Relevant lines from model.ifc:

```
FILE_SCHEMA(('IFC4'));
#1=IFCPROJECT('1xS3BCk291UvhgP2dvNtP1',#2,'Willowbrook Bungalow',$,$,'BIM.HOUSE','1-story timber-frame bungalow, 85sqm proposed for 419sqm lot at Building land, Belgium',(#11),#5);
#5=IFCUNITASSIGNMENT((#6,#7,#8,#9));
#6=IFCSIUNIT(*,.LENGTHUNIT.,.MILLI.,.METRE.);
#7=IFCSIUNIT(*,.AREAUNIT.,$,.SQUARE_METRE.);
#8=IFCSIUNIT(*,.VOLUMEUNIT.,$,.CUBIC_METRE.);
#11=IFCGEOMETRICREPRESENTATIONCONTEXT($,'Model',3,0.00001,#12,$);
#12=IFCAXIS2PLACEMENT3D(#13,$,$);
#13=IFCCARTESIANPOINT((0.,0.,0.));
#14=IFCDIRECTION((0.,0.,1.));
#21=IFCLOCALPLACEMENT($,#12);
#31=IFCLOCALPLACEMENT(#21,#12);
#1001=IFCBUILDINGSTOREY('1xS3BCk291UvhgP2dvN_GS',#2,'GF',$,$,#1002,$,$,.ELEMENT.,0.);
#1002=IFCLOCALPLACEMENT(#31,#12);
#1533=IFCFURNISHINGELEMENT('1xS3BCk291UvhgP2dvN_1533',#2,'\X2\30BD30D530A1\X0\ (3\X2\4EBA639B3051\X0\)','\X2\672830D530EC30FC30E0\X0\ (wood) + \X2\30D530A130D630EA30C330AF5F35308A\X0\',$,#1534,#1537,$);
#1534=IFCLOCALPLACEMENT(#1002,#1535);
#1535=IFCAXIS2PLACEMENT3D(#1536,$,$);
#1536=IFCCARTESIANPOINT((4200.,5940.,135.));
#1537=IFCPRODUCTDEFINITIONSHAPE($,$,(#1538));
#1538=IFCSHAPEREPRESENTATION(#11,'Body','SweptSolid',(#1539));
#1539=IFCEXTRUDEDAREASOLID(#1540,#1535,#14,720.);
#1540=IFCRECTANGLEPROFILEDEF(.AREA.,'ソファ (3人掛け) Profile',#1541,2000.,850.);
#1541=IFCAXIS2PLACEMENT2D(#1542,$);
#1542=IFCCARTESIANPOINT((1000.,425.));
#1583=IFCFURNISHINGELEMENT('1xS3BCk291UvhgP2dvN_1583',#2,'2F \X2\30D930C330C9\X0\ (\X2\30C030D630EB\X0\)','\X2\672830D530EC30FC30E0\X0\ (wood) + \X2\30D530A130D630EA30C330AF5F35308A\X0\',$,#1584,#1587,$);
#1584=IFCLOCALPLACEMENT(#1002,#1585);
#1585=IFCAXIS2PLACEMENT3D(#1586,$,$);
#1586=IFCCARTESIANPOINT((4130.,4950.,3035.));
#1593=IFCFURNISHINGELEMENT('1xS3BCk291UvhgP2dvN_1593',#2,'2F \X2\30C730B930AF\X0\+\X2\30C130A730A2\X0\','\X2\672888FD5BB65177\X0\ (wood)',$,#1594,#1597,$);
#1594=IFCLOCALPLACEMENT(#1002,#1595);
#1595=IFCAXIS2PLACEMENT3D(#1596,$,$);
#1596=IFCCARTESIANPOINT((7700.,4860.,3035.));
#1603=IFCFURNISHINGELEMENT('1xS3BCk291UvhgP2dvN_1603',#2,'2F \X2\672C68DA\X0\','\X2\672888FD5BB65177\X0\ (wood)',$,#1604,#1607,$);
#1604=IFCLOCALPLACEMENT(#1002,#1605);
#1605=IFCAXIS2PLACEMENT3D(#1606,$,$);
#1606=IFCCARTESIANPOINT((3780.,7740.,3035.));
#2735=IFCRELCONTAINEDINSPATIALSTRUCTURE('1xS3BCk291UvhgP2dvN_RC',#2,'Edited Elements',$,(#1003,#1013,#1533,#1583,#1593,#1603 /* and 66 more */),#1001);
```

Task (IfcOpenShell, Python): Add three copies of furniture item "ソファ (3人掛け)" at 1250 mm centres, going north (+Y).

```python
import numpy as np
import ifcopenshell
import ifcopenshell.api.geometry
import ifcopenshell.api.root
import ifcopenshell.util.element
import ifcopenshell.util.placement
import ifcopenshell.util.unit

model = ifcopenshell.open("model.ifc")
unit_scale = ifcopenshell.util.unit.calculate_unit_scale(model)


def reuse_history(source, copy):
    """copy_class also copies each property set's owner history, people and application; keep the originals."""
    for rel in copy.IsDefinedBy:
        if rel.is_a("IfcRelDefinesByProperties") and (history := rel.RelatingPropertyDefinition.OwnerHistory):
            rel.RelatingPropertyDefinition.OwnerHistory = source.OwnerHistory
            ifcopenshell.util.element.remove_deep2(model, history)


source = model.by_guid("1xS3BCk291UvhgP2dvN_1533")
base = ifcopenshell.util.placement.get_local_placement(source.ObjectPlacement)
step = np.array([0.0, 1.0, 0.0]) * 1.25 / unit_scale

for i in range(1, 4):
    copy = ifcopenshell.api.root.copy_class(model, product=source)
    copy.Representation = ifcopenshell.util.element.copy_deep(
        model, source.Representation, exclude=["IfcGeometricRepresentationContext", "IfcRepresentationMap"]
    )
    reuse_history(source, copy)
    matrix = base.copy()
    matrix[:3, 3] += i * step
    print("added at", matrix[:3, 3].round(3) + 0.0)
    ifcopenshell.api.geometry.edit_object_placement(model, product=copy, matrix=matrix, is_si=False)

model.write("model_edited.ifc")
```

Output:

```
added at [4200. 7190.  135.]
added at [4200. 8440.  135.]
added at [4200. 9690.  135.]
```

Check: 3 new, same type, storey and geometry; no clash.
